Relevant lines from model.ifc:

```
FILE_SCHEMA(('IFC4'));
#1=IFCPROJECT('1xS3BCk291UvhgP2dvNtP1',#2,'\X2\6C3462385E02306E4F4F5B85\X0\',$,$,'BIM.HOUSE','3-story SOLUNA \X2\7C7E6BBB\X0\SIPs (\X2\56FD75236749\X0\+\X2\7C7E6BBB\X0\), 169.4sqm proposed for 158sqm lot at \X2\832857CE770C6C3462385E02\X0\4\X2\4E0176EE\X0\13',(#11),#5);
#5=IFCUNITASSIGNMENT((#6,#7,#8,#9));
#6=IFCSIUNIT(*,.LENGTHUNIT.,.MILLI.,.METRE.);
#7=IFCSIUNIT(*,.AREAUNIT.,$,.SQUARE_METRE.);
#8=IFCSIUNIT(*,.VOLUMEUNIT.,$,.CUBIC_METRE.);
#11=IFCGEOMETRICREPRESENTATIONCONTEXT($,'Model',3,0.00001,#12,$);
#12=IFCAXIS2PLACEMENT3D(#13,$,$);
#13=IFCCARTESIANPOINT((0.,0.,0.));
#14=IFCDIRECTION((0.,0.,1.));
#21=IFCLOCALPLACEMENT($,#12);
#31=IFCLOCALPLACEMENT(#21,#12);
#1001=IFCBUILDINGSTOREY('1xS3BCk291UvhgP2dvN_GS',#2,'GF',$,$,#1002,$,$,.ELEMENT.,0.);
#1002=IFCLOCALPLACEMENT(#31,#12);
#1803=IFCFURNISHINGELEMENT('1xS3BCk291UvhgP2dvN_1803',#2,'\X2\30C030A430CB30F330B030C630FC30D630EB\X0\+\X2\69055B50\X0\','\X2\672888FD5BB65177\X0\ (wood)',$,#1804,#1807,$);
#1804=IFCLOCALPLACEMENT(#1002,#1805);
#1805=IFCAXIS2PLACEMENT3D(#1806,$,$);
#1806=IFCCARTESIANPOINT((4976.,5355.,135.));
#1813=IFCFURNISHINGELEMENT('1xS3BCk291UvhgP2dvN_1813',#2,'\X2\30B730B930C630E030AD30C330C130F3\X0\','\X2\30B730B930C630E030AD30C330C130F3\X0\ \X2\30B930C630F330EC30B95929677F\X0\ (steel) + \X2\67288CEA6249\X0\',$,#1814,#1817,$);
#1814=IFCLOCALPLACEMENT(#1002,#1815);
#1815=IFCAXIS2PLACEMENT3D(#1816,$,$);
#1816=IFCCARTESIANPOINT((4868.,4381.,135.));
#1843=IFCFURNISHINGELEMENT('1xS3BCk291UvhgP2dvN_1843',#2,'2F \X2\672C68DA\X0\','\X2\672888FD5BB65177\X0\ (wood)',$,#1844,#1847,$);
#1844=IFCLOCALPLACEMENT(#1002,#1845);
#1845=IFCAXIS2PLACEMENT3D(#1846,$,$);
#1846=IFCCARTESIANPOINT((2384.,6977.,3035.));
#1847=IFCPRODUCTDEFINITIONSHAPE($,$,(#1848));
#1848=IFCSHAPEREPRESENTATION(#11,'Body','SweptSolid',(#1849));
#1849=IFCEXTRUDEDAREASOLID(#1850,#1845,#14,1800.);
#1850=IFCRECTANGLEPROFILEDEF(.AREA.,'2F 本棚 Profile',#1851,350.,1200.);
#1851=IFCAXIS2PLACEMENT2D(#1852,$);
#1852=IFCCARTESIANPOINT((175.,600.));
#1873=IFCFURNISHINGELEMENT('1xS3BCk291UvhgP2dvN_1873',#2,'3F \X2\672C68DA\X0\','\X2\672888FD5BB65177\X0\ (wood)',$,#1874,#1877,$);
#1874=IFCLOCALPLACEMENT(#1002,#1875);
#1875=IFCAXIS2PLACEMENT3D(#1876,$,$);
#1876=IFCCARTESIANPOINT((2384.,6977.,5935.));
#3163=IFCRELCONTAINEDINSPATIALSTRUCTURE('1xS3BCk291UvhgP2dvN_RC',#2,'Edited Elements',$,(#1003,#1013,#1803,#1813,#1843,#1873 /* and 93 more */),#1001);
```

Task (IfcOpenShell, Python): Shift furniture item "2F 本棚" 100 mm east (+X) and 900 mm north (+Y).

```python
import ifcopenshell
import ifcopenshell.api.geometry
import ifcopenshell.util.placement

model = ifcopenshell.open("model.ifc")

item = model.by_guid("1xS3BCk291UvhgP2dvN_1843")
matrix = ifcopenshell.util.placement.get_local_placement(item.ObjectPlacement)
matrix[0, 3] += 100.0
matrix[1, 3] += 900.0
ifcopenshell.api.geometry.edit_object_placement(model, product=item, matrix=matrix, is_si=False)

print(ifcopenshell.util.placement.get_local_placement(item.ObjectPlacement).round(3) + 0.0)

model.write("model_edited.ifc")
```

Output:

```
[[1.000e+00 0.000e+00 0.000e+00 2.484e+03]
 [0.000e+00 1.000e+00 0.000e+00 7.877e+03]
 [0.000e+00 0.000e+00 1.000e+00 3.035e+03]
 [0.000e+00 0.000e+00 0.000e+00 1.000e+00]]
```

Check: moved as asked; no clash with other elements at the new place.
